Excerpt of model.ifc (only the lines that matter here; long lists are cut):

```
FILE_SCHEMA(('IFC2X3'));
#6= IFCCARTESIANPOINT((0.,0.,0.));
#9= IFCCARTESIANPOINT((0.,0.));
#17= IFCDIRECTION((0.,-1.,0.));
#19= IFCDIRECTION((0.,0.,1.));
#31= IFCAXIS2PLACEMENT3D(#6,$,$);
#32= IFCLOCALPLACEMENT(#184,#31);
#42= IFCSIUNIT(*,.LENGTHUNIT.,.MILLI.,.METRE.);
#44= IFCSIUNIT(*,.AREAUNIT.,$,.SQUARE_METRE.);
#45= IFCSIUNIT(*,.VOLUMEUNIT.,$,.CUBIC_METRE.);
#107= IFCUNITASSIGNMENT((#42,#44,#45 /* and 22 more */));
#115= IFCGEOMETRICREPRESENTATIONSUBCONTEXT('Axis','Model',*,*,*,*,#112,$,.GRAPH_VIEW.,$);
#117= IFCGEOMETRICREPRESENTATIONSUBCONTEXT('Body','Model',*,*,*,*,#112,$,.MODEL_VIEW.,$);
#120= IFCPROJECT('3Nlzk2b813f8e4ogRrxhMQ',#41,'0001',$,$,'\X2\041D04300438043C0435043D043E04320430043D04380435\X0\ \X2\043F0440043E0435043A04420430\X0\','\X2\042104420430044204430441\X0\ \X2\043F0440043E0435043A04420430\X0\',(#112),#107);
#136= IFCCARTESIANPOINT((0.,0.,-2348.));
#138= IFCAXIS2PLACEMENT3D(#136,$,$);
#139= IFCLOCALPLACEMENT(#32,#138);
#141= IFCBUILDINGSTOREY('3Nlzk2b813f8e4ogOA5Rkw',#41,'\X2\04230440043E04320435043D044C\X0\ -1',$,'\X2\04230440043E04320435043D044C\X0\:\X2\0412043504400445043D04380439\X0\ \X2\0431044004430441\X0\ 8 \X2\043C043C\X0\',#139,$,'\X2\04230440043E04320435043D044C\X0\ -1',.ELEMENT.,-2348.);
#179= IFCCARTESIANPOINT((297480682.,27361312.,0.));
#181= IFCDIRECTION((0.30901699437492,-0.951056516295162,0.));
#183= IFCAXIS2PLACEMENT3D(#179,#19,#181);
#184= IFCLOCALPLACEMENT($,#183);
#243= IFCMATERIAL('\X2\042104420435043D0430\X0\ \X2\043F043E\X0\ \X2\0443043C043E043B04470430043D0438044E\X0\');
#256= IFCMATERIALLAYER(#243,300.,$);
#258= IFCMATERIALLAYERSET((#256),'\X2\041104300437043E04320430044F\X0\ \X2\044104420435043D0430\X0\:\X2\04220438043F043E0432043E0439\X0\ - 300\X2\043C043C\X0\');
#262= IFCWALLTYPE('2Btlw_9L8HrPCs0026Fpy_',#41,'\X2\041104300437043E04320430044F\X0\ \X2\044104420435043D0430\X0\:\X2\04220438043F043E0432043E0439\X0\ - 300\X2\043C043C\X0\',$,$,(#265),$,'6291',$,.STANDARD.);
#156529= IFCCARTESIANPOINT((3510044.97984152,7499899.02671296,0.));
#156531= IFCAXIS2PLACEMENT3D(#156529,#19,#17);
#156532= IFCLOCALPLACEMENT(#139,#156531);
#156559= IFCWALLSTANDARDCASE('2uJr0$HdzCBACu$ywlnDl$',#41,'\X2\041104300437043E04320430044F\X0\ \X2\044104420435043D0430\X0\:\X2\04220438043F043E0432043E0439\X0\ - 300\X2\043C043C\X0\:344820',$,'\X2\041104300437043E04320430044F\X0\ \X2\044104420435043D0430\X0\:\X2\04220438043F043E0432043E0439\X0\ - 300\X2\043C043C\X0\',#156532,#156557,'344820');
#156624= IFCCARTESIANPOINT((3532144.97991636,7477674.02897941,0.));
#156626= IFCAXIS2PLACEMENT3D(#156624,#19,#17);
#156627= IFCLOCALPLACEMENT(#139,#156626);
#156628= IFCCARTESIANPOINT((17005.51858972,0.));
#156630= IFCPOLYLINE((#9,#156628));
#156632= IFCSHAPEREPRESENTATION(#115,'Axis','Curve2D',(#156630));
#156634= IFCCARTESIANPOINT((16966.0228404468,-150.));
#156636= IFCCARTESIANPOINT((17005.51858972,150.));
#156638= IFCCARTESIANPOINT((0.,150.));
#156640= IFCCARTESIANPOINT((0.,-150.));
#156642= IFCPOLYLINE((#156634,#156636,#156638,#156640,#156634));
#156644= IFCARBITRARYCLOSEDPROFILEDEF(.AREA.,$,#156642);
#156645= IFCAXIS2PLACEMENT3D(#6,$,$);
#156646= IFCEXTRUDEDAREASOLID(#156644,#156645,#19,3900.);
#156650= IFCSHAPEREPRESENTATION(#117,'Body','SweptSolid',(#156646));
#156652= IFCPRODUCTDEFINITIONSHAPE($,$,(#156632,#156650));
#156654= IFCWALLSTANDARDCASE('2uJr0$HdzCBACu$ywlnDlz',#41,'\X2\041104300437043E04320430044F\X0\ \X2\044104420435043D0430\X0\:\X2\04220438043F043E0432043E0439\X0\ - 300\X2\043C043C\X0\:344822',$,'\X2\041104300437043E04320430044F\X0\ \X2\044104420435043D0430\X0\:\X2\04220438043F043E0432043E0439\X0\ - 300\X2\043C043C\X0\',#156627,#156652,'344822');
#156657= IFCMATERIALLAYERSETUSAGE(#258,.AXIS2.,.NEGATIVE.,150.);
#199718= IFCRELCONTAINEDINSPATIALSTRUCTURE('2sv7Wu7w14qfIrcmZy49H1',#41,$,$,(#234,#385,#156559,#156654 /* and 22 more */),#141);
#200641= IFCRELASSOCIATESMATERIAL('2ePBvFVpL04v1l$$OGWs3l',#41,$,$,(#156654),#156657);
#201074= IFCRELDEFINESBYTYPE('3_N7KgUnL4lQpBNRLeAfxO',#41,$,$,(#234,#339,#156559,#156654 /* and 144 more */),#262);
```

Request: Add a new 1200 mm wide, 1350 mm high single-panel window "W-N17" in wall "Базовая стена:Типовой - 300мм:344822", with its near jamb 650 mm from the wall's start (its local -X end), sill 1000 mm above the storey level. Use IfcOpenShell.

```python
import numpy as np
import ifcopenshell
import ifcopenshell.api.feature
import ifcopenshell.api.geometry
import ifcopenshell.api.root
import ifcopenshell.api.spatial
import ifcopenshell.api.type
import ifcopenshell.geom
import ifcopenshell.util.element
import ifcopenshell.util.placement
import ifcopenshell.util.representation
import ifcopenshell.util.shape
import ifcopenshell.util.unit

model = ifcopenshell.open("model.ifc")
unit_scale = ifcopenshell.util.unit.calculate_unit_scale(model)
settings = ifcopenshell.geom.settings()


def volume(element):
    """Net volume in cubic metres, openings subtracted."""
    shape = ifcopenshell.geom.create_shape(settings, element)
    return ifcopenshell.util.shape.get_volume(shape.geometry)


wall = model.by_guid("2uJr0$HdzCBACu$ywlnDlz")
storey = ifcopenshell.util.element.get_container(wall, ifc_class="IfcBuildingStorey")
context = ifcopenshell.util.representation.get_context(model, "Model", "Body", "MODEL_VIEW")
before = volume(wall)

width, height, from_end, sill = 1.2, 1.35, 0.65, 1  # metres

# The wall runs along its own X axis, and the end named is its -X end.
wall_shape = ifcopenshell.geom.create_shape(settings, wall)
x, y, z = ifcopenshell.util.shape.get_vertices(wall_shape.geometry).T
start = x.min() + from_end
face, thickness = float(y.min()), float(y.max() - y.min())
wall_matrix = ifcopenshell.util.placement.get_local_placement(wall.ObjectPlacement)
level = ifcopenshell.util.placement.get_local_placement(storey.ObjectPlacement)[2, 3]


def in_wall(x, y):
    """Placement at x, y metres in the wall's axes, at sill height."""
    matrix = wall_matrix.copy()
    matrix[:, 3] = wall_matrix @ np.array([x / unit_scale, y / unit_scale, 0.0, 1.0])
    matrix[2, 3] = level + sill / unit_scale
    return matrix


# Opening: a box that overshoots both wall faces by 50 mm.
opening = ifcopenshell.api.root.create_entity(model, ifc_class="IfcOpeningElement")
box = ifcopenshell.api.geometry.add_wall_representation(
    model, context=context, length=width, height=height, thickness=thickness + 0.1
)
ifcopenshell.api.geometry.assign_representation(model, product=opening, representation=box)
ifcopenshell.api.geometry.edit_object_placement(model, product=opening, matrix=in_wall(start, face - 0.05), is_si=False)
ifcopenshell.api.feature.add_feature(model, feature=opening, element=wall)

window = ifcopenshell.api.root.create_entity(model, ifc_class="IfcWindow", name="W-N17")
window.OverallWidth, window.OverallHeight = width / unit_scale, height / unit_scale
body = ifcopenshell.api.geometry.add_window_representation(
    model,
    context=context,
    overall_width=window.OverallWidth,
    overall_height=window.OverallHeight,
    partition_type="SINGLE_PANEL",
)
ifcopenshell.api.geometry.assign_representation(model, product=window, representation=body)
ifcopenshell.api.spatial.assign_container(model, products=[window], relating_structure=storey)
fills = ifcopenshell.api.feature.add_filling(model, opening=opening, element=window)
fills.OwnerHistory = window.OwnerHistory  # required in IFC2X3

# IFC2X3 keeps the operation on the window style.
style = ifcopenshell.api.root.create_entity(model, ifc_class="IfcWindowStyle", name="W-N17")
style.OperationType, style.ConstructionType = "SINGLE_PANEL", "NOTDEFINED"
style.ParameterTakesPrecedence = style.Sizeable = False
ifcopenshell.api.type.assign_type(model, related_objects=[window], relating_type=style)

# Centre the window in the wall's thickness.
ifcopenshell.api.geometry.edit_object_placement(model, product=window, matrix=in_wall(start, face), is_si=False)
window_shape = ifcopenshell.geom.create_shape(settings, window)
depth = ifcopenshell.util.shape.get_vertices(window_shape.geometry)[:, 1]
offset = face + thickness / 2 - (depth.min() + depth.max()) / 2
ifcopenshell.api.geometry.edit_object_placement(model, product=window, matrix=in_wall(start, offset), is_si=False)

after = volume(wall)

print(f"wall volume {before:.3f} -> {after:.3f} m3")

model.write("model_rev.ifc")
```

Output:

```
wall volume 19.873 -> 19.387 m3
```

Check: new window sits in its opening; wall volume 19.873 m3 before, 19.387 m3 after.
